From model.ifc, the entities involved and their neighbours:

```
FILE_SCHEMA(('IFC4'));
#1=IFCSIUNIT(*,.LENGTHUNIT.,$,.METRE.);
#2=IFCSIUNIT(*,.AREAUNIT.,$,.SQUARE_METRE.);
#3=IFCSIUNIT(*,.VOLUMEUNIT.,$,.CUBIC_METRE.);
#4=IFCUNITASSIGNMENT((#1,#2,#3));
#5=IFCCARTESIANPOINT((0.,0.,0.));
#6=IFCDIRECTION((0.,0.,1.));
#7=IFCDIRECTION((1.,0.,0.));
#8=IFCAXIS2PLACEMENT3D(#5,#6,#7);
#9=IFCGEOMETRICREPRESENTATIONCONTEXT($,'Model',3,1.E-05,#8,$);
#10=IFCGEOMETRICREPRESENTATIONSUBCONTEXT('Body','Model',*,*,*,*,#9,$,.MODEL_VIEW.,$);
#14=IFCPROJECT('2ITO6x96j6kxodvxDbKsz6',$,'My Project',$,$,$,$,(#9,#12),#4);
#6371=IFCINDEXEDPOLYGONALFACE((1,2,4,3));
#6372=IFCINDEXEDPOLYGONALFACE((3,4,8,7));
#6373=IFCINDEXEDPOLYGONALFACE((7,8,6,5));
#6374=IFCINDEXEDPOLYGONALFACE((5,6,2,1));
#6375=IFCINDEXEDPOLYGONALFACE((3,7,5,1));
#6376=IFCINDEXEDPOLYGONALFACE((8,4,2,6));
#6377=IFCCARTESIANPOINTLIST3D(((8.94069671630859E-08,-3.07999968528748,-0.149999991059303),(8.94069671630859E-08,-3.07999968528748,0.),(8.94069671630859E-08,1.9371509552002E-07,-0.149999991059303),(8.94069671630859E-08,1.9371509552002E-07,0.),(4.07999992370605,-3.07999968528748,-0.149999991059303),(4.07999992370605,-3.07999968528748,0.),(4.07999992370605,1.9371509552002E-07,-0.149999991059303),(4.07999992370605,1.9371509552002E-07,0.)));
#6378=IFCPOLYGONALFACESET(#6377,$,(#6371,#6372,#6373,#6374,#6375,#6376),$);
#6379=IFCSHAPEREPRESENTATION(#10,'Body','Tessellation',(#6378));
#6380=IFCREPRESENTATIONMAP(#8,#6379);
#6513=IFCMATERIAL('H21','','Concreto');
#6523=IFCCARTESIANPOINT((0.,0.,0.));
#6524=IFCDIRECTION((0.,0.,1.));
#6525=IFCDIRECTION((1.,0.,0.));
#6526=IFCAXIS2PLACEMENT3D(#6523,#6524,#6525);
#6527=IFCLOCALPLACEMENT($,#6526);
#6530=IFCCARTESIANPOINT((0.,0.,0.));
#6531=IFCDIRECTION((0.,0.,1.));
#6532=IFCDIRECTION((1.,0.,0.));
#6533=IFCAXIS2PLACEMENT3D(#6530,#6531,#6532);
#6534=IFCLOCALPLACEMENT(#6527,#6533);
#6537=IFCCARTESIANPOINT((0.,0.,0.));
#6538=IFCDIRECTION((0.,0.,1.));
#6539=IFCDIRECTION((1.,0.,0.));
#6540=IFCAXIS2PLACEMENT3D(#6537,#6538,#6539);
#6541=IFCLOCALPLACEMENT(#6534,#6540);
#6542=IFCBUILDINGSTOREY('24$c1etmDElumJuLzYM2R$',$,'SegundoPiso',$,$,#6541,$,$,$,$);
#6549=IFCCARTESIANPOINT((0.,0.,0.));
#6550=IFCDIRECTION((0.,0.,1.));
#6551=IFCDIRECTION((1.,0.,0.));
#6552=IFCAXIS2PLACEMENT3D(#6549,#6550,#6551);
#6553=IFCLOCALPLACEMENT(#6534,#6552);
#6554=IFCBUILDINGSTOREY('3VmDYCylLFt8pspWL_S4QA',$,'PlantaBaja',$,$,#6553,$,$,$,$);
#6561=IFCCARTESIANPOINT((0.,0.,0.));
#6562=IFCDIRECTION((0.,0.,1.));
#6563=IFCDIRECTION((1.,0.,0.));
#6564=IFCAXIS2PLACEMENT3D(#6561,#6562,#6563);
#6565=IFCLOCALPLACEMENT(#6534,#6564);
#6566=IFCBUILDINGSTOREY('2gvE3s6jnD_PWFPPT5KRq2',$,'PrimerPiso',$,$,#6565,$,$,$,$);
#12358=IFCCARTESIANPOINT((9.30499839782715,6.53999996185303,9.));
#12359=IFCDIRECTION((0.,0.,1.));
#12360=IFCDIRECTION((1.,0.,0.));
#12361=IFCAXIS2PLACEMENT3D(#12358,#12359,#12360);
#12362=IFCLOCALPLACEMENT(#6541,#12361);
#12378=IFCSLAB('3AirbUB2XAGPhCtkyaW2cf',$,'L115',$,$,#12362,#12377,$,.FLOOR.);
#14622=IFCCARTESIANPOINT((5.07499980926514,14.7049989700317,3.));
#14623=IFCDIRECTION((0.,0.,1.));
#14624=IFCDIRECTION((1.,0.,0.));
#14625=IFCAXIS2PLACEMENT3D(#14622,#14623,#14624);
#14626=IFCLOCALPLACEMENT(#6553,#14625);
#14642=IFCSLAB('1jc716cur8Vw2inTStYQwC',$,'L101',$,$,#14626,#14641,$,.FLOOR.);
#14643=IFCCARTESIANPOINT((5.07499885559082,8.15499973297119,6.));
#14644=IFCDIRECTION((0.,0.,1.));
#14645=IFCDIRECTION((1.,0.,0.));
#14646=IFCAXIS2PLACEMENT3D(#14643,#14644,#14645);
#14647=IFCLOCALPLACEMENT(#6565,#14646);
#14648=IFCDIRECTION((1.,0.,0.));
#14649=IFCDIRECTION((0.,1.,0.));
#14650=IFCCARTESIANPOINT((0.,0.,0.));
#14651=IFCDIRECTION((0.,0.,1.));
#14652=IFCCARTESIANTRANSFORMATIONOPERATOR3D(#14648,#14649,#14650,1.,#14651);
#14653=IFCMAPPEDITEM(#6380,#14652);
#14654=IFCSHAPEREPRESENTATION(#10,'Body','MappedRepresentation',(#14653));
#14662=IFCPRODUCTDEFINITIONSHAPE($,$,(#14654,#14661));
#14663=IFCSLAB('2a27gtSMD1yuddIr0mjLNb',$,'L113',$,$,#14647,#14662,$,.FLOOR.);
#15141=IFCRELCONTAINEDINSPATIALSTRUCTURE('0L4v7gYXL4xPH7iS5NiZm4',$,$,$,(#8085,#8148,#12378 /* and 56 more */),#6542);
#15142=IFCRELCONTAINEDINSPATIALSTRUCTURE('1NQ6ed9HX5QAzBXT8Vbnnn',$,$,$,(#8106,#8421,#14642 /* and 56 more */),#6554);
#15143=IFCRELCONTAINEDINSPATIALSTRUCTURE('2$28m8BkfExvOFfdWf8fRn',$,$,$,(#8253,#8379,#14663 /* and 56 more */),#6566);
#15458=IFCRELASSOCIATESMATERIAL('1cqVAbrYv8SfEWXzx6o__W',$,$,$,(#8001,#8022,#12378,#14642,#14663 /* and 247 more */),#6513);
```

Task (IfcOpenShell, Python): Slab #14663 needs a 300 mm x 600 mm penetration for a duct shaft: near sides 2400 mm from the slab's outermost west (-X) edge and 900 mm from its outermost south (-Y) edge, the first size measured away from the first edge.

```python
import numpy as np
import ifcopenshell
import ifcopenshell.api.feature
import ifcopenshell.api.geometry
import ifcopenshell.api.root
import ifcopenshell.geom
import ifcopenshell.util.placement
import ifcopenshell.util.representation
import ifcopenshell.util.shape
import ifcopenshell.util.unit

model = ifcopenshell.open("model.ifc")
unit_scale = ifcopenshell.util.unit.calculate_unit_scale(model)
settings = ifcopenshell.geom.settings()


def volume(element):
    """Net volume in cubic metres, openings subtracted."""
    shape = ifcopenshell.geom.create_shape(settings, element)
    return ifcopenshell.util.shape.get_volume(shape.geometry)


slab = model.by_guid("2a27gtSMD1yuddIr0mjLNb")
before = volume(slab)

# Extent in the slab's own axes, in metres. The edges named are its -X and -Y sides.
slab_shape = ifcopenshell.geom.create_shape(settings, slab)
vertices = ifcopenshell.util.shape.get_vertices(slab_shape.geometry)
x_min, y_min, bottom = vertices.min(axis=0)
top = vertices[:, 2].max()

opening = ifcopenshell.api.root.create_entity(model, ifc_class="IfcOpeningElement", name="Duct shaft opening", predefined_type="OPENING")
context = ifcopenshell.util.representation.get_context(model, "Model", "Body", "MODEL_VIEW")
width, depth = 0.3, 0.6
outline = [(0.0, 0.0), (width, 0.0), (width, depth), (0.0, depth), (0.0, 0.0)]
# Overshoot both faces by 50 mm so the cut is clean.
shape = ifcopenshell.api.geometry.add_slab_representation(
    model, context=context, depth=top - bottom + 0.1, polyline=outline
)
ifcopenshell.api.geometry.assign_representation(model, product=opening, representation=shape)

matrix = ifcopenshell.util.placement.get_local_placement(slab.ObjectPlacement)
matrix[:, 3] = matrix @ np.append(np.array([x_min + 2.4, y_min + 0.9, bottom - 0.05]) / unit_scale, 1.0)
ifcopenshell.api.geometry.edit_object_placement(model, product=opening, matrix=matrix, is_si=False)
ifcopenshell.api.feature.add_feature(model, feature=opening, element=slab)

after = volume(slab)

print(f"slab volume {before:.3f} -> {after:.3f} m3")

model.write("model_edited.ifc")
```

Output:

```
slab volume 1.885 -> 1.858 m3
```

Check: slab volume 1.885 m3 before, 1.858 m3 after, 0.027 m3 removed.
